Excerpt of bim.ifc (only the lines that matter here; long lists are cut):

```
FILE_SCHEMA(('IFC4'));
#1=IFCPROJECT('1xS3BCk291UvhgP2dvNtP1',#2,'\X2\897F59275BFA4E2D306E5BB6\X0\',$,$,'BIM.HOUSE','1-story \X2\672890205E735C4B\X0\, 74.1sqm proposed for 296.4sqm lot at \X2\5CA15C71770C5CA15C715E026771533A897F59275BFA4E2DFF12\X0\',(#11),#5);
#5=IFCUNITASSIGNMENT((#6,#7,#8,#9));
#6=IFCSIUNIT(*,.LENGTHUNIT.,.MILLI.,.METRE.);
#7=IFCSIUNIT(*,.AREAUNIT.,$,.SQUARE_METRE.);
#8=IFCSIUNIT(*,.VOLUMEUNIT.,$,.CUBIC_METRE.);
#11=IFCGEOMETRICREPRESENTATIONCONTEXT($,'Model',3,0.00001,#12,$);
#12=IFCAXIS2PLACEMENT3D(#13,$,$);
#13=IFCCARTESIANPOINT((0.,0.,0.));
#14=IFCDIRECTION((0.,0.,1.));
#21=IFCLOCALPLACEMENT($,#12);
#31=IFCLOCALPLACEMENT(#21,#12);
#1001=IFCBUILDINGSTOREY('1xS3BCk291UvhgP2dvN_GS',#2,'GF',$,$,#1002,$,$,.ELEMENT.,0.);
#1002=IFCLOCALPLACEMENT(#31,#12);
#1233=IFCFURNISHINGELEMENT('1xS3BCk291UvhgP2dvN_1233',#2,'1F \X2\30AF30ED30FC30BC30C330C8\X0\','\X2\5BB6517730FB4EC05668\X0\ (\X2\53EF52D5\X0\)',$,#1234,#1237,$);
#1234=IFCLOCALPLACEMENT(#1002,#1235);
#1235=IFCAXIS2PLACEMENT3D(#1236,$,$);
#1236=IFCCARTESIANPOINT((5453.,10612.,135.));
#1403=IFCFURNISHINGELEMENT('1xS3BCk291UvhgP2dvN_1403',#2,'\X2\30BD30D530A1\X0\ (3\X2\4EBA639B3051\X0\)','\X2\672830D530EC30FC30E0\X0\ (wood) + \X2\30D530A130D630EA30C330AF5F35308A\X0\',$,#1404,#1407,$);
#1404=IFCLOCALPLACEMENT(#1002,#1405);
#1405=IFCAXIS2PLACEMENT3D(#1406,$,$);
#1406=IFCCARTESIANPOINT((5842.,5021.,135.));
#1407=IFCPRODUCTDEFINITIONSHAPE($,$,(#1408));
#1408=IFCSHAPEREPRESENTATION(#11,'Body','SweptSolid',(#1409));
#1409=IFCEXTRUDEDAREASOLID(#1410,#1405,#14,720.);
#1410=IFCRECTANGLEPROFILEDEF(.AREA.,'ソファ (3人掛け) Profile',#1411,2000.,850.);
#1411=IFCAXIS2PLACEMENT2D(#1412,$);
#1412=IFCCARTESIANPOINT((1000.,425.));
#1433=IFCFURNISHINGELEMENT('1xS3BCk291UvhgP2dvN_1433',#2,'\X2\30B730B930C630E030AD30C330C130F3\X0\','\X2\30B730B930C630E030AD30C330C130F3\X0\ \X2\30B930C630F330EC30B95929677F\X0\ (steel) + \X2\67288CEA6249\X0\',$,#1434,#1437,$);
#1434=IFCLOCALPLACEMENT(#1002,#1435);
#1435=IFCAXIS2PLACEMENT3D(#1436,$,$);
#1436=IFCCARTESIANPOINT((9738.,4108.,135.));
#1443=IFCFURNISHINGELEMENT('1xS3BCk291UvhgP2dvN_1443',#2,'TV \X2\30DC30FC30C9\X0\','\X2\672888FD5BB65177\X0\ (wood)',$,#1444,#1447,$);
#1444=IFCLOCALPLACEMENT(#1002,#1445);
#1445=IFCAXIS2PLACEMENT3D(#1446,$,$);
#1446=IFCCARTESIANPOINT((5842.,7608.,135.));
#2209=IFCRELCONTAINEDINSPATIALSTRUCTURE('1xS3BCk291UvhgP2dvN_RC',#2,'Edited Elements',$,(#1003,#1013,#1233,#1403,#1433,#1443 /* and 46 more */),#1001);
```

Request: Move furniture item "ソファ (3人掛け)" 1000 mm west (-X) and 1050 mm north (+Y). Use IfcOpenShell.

```python
import ifcopenshell
import ifcopenshell.api.geometry
import ifcopenshell.util.placement
import ifcopenshell.util.unit

model = ifcopenshell.open("bim.ifc")
unit_scale = ifcopenshell.util.unit.calculate_unit_scale(model)

item = model.by_guid("1xS3BCk291UvhgP2dvN_1403")
matrix = ifcopenshell.util.placement.get_local_placement(item.ObjectPlacement)
matrix[0, 3] -= 1 / unit_scale
matrix[1, 3] += 1.05 / unit_scale
ifcopenshell.api.geometry.edit_object_placement(model, product=item, matrix=matrix, is_si=False)

print(ifcopenshell.util.placement.get_local_placement(item.ObjectPlacement).round(3) + 0.0)

model.write("bim-out.ifc")
```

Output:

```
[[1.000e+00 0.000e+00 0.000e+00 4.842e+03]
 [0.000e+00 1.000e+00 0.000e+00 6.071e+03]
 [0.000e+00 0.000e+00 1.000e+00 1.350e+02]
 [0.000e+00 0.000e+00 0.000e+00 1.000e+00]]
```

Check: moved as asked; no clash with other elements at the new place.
